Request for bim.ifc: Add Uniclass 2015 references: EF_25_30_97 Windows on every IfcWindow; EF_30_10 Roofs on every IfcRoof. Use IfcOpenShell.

First a look at what the model holds.

```python
import ifcopenshell

model = ifcopenshell.open("bim.ifc")
print(model.schema)
print("classifications:", [c.Name for c in model.by_type("IfcClassification")])
for ifc_class in ("IfcDoor", "IfcRoof", "IfcStair", "IfcWall", "IfcWindow"):
    print(ifc_class, len(model.by_type(ifc_class)))
```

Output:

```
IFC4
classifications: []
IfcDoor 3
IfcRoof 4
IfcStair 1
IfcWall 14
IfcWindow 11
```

```python
import ifcopenshell
import ifcopenshell.api.classification

model = ifcopenshell.open("bim.ifc")

system = ifcopenshell.api.classification.add_classification(model, classification="Uniclass 2015")

codes = {
    "IfcWindow": ("EF_25_30_97", "Windows"),
    "IfcRoof": ("EF_30_10", "Roofs"),
}
for ifc_class, (code, name) in codes.items():
    products = model.by_type(ifc_class)
    ifcopenshell.api.classification.add_reference(
        model, products=products, classification=system, identification=code, name=name
    )
    print(code, len(products))

model.write("bim_updated.ifc")
```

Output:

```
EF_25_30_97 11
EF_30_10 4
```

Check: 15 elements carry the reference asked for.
